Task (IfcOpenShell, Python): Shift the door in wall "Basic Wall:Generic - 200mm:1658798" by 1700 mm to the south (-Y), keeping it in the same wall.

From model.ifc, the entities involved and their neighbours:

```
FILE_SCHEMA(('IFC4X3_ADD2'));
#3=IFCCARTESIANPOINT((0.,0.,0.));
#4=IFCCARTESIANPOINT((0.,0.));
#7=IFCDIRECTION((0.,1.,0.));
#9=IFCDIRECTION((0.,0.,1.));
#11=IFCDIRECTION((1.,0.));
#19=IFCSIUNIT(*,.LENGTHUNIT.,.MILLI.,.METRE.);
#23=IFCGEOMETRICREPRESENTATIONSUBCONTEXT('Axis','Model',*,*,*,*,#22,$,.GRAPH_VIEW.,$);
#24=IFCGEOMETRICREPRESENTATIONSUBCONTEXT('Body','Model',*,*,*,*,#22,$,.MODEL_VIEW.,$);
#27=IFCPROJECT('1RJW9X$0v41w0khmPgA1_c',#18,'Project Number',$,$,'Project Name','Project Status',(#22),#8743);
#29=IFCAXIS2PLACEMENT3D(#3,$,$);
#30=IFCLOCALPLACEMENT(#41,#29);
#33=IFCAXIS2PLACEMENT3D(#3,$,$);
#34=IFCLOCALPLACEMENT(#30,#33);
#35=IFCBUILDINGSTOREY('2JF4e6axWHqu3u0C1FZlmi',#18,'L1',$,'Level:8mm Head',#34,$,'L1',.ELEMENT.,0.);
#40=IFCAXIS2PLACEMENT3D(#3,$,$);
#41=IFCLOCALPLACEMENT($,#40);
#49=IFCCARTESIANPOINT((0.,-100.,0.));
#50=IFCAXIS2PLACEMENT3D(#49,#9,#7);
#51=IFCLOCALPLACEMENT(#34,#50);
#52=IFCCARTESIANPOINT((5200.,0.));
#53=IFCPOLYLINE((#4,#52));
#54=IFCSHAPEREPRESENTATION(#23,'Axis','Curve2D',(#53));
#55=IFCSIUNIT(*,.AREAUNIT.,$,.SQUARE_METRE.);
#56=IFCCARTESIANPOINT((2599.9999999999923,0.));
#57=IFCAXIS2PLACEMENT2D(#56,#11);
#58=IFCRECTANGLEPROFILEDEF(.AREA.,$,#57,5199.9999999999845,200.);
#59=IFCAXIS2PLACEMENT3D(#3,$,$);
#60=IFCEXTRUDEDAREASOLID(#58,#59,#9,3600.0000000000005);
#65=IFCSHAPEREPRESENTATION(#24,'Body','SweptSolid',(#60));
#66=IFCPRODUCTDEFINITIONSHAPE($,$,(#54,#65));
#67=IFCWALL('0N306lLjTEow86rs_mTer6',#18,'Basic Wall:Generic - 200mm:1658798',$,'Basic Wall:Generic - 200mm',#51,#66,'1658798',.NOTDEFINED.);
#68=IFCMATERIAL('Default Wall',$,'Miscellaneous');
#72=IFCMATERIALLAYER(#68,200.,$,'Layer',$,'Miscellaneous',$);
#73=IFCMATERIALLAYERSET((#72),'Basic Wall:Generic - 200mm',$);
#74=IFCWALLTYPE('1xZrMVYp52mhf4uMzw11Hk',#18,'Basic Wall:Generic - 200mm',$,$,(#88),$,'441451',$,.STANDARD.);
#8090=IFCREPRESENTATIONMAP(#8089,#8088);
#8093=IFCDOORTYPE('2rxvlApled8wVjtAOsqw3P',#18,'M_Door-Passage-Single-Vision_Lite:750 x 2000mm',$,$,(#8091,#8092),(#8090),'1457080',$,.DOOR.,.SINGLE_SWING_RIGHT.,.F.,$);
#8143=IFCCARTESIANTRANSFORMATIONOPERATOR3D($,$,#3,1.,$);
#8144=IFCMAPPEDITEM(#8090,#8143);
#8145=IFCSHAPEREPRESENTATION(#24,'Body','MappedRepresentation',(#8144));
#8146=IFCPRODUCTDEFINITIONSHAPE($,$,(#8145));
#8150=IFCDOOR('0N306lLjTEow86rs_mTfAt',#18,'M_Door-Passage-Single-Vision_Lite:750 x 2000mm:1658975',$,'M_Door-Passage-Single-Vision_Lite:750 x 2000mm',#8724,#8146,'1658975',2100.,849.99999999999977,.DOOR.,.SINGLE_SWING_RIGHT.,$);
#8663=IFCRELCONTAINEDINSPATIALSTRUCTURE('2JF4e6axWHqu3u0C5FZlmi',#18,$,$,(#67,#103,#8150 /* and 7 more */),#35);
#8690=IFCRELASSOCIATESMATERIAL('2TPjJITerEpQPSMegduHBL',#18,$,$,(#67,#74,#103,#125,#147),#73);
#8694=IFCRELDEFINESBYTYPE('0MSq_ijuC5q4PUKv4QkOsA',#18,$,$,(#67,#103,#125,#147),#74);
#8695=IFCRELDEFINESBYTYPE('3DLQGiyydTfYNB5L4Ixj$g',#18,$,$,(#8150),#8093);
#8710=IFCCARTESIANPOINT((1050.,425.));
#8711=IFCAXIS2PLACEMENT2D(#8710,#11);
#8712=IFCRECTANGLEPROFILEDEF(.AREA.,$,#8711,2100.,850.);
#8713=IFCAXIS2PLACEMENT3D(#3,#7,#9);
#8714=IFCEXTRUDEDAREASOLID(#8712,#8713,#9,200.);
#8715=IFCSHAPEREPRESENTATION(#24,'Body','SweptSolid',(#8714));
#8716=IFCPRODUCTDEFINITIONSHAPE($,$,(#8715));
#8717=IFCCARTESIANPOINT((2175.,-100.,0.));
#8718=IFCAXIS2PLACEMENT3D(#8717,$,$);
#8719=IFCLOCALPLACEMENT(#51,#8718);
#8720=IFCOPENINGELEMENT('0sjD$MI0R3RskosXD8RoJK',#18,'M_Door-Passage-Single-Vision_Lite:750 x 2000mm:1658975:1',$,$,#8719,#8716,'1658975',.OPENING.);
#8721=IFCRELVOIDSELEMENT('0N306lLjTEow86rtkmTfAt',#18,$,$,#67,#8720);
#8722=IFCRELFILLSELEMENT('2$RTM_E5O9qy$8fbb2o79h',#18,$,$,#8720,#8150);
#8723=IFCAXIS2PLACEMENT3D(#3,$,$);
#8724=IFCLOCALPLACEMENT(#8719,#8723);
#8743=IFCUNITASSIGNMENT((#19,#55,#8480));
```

```python
import ifcopenshell
import ifcopenshell.api.geometry
import ifcopenshell.util.placement
import ifcopenshell.util.unit

model = ifcopenshell.open("model.ifc")
unit_scale = ifcopenshell.util.unit.calculate_unit_scale(model)

door = model.by_guid("0N306lLjTEow86rs_mTfAt")
opening = door.FillsVoids[0].RelatingOpeningElement
wall = opening.VoidsElements[0].RelatingBuildingElement

wall_matrix = ifcopenshell.util.placement.get_local_placement(wall.ObjectPlacement)
shift = wall_matrix[:3, 0] * -1.7 / unit_scale
before = ifcopenshell.util.placement.get_local_placement(door.ObjectPlacement)[:3, 3].copy()

# The door is placed relative to its opening, so it follows when the opening moves.
matrix = ifcopenshell.util.placement.get_local_placement(opening.ObjectPlacement)
matrix[:3, 3] += shift
ifcopenshell.api.geometry.edit_object_placement(
    model, product=opening, matrix=matrix, is_si=False, should_transform_children=True
)

after = ifcopenshell.util.placement.get_local_placement(door.ObjectPlacement)[:3, 3]
print("door moved by", (after - before).round(3) + 0.0)

model.write("model_updated.ifc")
```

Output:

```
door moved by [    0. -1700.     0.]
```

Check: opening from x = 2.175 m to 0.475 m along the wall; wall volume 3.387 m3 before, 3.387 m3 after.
